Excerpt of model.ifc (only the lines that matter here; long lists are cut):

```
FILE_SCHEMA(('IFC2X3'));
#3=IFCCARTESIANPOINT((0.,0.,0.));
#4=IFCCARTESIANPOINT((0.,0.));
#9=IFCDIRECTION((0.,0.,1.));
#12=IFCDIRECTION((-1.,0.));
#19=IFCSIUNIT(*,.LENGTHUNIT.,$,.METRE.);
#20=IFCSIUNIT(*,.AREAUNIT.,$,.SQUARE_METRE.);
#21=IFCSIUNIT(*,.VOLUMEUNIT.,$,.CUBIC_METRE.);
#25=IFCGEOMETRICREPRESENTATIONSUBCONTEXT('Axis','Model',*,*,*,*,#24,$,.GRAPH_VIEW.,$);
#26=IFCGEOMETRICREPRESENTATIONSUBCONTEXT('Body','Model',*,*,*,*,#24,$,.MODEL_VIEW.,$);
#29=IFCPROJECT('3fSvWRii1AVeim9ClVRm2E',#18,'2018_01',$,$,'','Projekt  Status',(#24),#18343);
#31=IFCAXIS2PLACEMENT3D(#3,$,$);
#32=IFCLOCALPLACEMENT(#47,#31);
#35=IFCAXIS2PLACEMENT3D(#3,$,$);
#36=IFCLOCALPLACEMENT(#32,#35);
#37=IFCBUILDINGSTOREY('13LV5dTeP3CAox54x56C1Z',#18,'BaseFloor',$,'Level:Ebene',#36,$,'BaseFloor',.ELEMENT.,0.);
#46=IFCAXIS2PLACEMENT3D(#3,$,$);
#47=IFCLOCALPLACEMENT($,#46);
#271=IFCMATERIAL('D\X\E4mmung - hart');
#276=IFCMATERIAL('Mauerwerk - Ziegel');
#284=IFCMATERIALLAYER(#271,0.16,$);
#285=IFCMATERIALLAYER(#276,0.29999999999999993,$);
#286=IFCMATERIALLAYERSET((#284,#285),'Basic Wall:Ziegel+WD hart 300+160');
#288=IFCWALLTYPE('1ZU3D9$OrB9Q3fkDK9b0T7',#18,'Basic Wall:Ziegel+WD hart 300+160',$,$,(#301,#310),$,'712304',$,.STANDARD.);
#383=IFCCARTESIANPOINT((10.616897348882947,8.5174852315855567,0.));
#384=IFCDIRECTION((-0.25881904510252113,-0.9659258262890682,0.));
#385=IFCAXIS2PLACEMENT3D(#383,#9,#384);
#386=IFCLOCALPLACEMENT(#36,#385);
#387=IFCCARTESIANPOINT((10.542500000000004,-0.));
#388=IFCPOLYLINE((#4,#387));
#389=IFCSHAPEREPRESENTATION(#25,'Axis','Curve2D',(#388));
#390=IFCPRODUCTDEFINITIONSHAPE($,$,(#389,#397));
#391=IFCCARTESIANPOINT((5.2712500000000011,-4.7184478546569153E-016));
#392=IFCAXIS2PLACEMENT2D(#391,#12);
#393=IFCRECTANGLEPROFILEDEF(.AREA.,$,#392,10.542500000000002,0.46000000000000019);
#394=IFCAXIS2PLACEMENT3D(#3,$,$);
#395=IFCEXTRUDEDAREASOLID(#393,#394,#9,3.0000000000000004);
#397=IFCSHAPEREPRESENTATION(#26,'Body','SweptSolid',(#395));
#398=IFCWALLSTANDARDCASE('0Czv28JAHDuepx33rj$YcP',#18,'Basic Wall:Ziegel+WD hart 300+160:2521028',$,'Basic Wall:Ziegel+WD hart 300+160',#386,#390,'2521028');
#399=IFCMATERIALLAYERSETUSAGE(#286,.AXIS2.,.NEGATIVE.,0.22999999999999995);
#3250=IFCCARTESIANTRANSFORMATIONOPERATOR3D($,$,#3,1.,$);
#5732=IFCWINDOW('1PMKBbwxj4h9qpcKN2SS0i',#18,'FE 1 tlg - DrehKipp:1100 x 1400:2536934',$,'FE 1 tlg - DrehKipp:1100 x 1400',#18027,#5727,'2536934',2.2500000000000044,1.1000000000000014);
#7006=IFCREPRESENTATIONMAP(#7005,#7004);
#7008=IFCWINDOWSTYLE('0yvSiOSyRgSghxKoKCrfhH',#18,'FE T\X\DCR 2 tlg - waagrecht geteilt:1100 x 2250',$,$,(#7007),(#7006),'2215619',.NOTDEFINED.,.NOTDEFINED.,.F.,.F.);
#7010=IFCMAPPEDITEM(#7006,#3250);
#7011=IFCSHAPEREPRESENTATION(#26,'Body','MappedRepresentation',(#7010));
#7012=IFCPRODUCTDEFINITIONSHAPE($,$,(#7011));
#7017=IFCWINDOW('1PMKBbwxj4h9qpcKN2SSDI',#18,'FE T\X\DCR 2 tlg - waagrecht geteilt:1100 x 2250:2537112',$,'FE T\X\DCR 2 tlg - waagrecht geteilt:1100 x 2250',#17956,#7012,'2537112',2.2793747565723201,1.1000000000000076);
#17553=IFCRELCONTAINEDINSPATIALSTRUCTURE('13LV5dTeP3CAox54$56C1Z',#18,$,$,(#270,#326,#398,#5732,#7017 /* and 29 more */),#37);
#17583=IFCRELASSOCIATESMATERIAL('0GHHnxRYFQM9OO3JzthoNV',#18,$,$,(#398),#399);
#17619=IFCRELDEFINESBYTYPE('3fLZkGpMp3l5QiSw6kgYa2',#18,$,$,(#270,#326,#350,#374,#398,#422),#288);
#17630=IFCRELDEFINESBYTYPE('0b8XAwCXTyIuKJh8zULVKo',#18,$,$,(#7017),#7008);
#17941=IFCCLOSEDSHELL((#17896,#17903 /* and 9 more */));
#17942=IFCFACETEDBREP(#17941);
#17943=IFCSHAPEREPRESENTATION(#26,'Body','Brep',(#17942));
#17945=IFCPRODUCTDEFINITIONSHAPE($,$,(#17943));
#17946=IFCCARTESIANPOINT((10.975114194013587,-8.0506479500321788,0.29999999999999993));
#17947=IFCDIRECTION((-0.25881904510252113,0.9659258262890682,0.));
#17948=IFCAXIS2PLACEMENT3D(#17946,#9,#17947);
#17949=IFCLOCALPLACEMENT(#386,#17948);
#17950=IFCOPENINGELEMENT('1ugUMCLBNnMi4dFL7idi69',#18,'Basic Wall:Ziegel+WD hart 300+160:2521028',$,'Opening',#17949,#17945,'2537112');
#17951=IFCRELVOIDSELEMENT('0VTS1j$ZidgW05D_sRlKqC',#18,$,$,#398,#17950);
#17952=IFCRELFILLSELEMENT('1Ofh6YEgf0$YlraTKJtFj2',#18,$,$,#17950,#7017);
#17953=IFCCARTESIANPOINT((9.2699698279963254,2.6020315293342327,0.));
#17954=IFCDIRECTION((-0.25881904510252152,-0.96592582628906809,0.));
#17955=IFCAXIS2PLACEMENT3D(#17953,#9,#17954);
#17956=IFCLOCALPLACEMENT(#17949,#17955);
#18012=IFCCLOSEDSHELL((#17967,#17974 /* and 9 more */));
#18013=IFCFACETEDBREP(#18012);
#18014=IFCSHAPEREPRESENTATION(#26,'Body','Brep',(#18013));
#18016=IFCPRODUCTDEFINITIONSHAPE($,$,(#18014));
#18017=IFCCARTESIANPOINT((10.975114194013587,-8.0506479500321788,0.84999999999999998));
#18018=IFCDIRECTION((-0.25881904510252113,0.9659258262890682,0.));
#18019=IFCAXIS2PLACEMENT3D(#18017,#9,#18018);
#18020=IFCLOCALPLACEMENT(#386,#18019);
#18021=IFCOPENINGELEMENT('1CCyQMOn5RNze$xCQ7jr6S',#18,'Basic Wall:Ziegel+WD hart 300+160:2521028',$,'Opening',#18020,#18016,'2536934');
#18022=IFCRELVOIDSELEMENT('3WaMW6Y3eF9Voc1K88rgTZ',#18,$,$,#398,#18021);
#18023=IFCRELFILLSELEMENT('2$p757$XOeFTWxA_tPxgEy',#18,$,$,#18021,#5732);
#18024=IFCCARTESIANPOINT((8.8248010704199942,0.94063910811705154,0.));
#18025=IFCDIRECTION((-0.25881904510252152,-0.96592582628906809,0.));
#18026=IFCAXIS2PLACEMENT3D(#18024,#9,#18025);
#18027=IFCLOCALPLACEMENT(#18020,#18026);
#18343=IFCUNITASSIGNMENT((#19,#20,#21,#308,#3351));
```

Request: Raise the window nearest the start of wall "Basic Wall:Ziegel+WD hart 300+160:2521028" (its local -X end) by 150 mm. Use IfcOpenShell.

```python
import numpy as np
import ifcopenshell
import ifcopenshell.api.geometry
import ifcopenshell.util.placement
import ifcopenshell.util.unit

model = ifcopenshell.open("model.ifc")
unit_scale = ifcopenshell.util.unit.calculate_unit_scale(model)

window = model.by_id(7017)
opening = window.FillsVoids[0].RelatingOpeningElement
dz = 0.15 / unit_scale

shift = np.array([0.0, 0.0, dz])
# The window is placed relative to its opening, so it follows when the opening moves.
matrix = ifcopenshell.util.placement.get_local_placement(opening.ObjectPlacement)
matrix[:3, 3] += shift
ifcopenshell.api.geometry.edit_object_placement(
    model, product=opening, matrix=matrix, is_si=False, should_transform_children=True
)

print(f"moved by {dz * unit_scale:+.3f} m")

model.write("model_v2.ifc")
```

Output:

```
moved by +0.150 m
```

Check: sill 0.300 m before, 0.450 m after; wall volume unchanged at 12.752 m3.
